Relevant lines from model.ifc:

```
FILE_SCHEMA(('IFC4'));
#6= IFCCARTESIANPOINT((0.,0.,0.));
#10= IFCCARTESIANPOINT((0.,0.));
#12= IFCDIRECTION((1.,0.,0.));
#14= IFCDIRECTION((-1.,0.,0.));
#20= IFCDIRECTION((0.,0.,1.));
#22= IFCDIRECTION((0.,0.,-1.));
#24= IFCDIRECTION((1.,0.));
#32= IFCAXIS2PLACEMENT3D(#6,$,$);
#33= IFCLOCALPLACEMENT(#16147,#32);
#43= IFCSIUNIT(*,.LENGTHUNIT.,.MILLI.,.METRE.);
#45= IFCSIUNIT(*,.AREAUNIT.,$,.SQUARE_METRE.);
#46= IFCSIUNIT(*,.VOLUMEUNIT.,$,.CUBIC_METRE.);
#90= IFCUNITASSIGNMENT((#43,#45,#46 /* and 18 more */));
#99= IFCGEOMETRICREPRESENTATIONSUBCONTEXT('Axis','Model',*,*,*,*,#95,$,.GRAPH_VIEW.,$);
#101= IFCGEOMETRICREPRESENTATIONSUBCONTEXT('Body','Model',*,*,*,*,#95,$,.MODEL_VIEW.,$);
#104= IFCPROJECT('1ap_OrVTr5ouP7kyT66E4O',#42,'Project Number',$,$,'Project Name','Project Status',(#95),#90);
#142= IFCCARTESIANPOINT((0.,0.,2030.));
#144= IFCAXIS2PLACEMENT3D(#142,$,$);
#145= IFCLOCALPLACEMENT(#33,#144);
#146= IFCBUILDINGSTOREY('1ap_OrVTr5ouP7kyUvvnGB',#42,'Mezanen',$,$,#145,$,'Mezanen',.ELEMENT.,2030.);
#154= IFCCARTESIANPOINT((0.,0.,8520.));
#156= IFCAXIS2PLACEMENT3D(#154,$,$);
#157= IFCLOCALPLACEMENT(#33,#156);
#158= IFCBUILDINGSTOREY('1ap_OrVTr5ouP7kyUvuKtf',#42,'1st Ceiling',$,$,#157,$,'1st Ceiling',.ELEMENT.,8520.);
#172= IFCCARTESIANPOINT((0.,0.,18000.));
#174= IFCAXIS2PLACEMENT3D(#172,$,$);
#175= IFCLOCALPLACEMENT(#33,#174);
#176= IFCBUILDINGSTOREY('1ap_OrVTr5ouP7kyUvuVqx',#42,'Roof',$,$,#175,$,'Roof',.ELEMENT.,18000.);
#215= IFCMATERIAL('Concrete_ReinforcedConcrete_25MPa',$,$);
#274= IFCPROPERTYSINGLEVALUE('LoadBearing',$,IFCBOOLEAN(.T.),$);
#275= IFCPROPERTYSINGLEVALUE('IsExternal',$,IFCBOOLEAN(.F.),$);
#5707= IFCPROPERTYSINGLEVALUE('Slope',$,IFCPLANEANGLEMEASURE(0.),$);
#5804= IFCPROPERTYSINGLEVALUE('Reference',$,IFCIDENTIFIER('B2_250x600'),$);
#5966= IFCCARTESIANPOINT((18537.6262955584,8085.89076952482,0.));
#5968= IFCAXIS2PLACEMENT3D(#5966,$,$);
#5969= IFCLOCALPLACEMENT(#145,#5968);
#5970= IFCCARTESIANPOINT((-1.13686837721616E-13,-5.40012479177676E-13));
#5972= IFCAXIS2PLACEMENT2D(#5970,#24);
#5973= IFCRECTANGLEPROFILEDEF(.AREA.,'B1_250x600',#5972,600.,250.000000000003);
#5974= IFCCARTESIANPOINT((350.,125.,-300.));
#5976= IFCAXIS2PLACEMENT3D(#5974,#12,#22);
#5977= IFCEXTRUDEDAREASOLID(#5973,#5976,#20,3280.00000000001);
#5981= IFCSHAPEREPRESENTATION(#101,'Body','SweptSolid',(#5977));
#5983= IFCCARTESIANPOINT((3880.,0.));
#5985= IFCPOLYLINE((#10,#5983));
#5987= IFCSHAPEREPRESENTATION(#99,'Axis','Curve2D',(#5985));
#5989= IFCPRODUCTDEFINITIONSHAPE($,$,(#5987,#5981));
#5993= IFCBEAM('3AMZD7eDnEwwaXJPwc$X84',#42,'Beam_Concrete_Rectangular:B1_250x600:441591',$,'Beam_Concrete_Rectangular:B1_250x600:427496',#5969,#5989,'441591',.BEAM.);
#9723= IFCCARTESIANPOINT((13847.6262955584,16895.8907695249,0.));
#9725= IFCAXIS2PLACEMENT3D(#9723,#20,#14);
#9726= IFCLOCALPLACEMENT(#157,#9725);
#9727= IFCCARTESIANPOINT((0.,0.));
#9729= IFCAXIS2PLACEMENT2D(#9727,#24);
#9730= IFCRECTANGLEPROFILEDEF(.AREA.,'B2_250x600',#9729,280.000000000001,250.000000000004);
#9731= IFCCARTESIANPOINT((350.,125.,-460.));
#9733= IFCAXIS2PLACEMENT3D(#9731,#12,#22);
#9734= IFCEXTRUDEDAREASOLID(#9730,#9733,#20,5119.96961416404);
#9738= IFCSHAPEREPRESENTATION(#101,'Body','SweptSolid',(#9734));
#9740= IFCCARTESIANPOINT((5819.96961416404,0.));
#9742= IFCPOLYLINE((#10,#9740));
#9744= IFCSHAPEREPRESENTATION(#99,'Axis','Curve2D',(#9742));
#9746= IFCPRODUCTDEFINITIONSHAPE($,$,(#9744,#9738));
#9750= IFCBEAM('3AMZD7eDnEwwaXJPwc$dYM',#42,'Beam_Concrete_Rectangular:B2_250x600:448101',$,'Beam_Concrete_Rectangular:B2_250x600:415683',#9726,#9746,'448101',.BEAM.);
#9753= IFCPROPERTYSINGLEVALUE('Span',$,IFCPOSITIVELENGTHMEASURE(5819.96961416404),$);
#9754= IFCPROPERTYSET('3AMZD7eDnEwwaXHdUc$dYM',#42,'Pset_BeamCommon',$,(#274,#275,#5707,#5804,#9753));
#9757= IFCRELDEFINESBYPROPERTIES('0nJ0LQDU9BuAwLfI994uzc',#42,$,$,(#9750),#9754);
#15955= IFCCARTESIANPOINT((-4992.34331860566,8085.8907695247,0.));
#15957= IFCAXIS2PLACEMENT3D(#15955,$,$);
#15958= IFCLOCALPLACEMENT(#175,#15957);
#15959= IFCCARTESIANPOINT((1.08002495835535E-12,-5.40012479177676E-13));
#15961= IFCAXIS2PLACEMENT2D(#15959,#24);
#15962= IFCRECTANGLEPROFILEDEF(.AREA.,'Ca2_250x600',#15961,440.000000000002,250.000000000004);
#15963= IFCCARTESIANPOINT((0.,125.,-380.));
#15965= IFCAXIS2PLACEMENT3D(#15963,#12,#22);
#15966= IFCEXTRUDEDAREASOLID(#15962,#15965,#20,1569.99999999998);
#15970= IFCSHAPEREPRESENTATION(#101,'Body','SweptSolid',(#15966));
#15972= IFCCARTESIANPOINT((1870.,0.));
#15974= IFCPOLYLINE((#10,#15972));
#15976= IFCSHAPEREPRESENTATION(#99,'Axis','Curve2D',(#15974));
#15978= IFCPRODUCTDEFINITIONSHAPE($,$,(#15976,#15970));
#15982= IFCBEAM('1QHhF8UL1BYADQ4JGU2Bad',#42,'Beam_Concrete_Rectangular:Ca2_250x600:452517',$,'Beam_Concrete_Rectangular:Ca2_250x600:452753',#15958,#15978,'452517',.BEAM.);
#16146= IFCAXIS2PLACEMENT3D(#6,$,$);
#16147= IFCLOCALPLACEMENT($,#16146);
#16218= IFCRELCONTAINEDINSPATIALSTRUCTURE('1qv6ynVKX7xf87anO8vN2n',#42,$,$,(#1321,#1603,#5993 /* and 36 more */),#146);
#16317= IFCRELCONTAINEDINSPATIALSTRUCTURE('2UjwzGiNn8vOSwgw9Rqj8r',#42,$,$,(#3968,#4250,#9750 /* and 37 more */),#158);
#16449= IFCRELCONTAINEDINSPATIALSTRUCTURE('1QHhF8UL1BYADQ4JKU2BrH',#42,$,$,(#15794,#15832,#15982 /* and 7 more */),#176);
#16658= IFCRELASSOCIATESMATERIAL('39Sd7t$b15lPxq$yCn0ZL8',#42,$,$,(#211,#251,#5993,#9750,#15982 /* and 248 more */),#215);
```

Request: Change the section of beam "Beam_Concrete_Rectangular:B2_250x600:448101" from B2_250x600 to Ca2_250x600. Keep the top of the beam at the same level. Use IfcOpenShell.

```python
import ifcopenshell
import ifcopenshell.api.pset
import ifcopenshell.util.element
import ifcopenshell.util.representation

model = ifcopenshell.open("model.ifc")

member = model.by_id(9750)
source = next(p for p in model.by_type("IfcRectangleProfileDef") if p.ProfileName == "Ca2_250x600")

body = ifcopenshell.util.representation.get_representation(member, "Model", "Body")
solid = body.Items[0]
old_profile = solid.SweptArea

# Copy the section's sizes but keep this member's own profile position.
profile = ifcopenshell.util.element.copy(model, source)
# Profiles are centred, so shift by half the change in depth to hold the top.
shift = (old_profile.XDim - profile.XDim) / 2
x, y = old_profile.Position.Location.Coordinates
up = (-1.0, 0.0)  # upwards, in the solid's own plane
location = model.createIfcCartesianPoint((x + up[0] * shift, y + up[1] * shift))
profile.Position = model.createIfcAxis2Placement2D(location, old_profile.Position.RefDirection)
solid.SweptArea = profile
if not model.get_total_inverses(old_profile):
    ifcopenshell.util.element.remove_deep2(model, old_profile)
member.Name = member.Name.replace("B2_250x600", "Ca2_250x600")
member.ObjectType = member.ObjectType.replace("B2_250x600", "Ca2_250x600")
pset = model.by_id(ifcopenshell.util.element.get_pset(member, "Pset_BeamCommon", should_inherit=False)["id"])
ifcopenshell.api.pset.edit_pset(model, pset=pset, properties={"Reference": "Ca2_250x600"})

print(solid.SweptArea)

model.write("model-out.ifc")
```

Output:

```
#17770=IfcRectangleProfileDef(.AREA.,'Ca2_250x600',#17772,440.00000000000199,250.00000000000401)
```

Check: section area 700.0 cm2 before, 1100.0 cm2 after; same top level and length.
